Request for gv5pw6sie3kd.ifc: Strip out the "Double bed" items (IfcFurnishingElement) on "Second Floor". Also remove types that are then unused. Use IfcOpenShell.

First a look at what the model holds.

```python
import ifcopenshell
import ifcopenshell.util.element

model = ifcopenshell.open("gv5pw6sie3kd.ifc")
print(model.schema)
storey = next(s for s in model.by_type("IfcBuildingStorey") if s.Name == "Second Floor")
furniture = [e for e in ifcopenshell.util.element.get_decomposition(storey) if e.is_a("IfcFurnishingElement")]
seen = {}
for e in furniture:
    element_type = ifcopenshell.util.element.get_type(e)
    name = element_type.Name if element_type not in (None, e) else None
    seen[name] = seen.get(name, 0) + 1
for name, count in sorted(seen.items(), key=str):
    print(count, "x", name)
```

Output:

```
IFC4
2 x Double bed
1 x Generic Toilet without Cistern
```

```python
import ifcopenshell
import ifcopenshell.api.root
import ifcopenshell.util.element

model = ifcopenshell.open("gv5pw6sie3kd.ifc")

storey = next(s for s in model.by_type("IfcBuildingStorey") if s.Name == "Second Floor")
furniture = [e for e in ifcopenshell.util.element.get_decomposition(storey) if e.is_a("IfcFurnishingElement")]
targets = [e for e in furniture if (t := ifcopenshell.util.element.get_type(e)) not in (None, e) and t.Name == "Double bed"]
types = {ifcopenshell.util.element.get_type(e) for e in targets} - {None, *targets}

for e in targets:
    ifcopenshell.api.root.remove_product(model, product=e)
print(len(targets), "removed")

unused = [t for t in types if not ifcopenshell.util.element.get_types(t)]
for t in unused:
    ifcopenshell.api.root.remove_product(model, product=t)
print(len(unused), "unused types removed")

model.write("gv5pw6sie3kd_updated.ifc")
```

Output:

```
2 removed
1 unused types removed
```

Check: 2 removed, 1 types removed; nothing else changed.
